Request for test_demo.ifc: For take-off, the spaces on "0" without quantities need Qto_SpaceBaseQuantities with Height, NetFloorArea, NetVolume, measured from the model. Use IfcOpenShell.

First a look at what the model holds.

```python
import ifcopenshell
import ifcopenshell.util.element
import ifcopenshell.util.unit

model = ifcopenshell.open("test_demo.ifc")
print(model.schema)
for unit_type in ("LENGTHUNIT", "AREAUNIT", "VOLUMEUNIT"):
    print(unit_type, ifcopenshell.util.unit.calculate_unit_scale(model, unit_type))
storey = next(s for s in model.by_type("IfcBuildingStorey") if s.Name == "0")
spaces = [e for e in ifcopenshell.util.element.get_decomposition(storey) if e.is_a("IfcSpace")]
for e in sorted(spaces, key=lambda e: e.id()):
    print(e.id(), e.is_a(), e.Name, list(ifcopenshell.util.element.get_psets(e, qtos_only=True)), sep=" | ")
```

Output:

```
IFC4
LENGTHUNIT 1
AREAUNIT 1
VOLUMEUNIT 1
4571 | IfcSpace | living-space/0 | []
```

```python
import ifcopenshell
import ifcopenshell.api.pset
import ifcopenshell.geom
import ifcopenshell.util.element
import ifcopenshell.util.shape
import ifcopenshell.util.unit

model = ifcopenshell.open("test_demo.ifc")
unit_scale = ifcopenshell.util.unit.calculate_unit_scale(model)
area_scale = ifcopenshell.util.unit.calculate_unit_scale(model, "AREAUNIT")
volume_scale = ifcopenshell.util.unit.calculate_unit_scale(model, "VOLUMEUNIT")
settings = ifcopenshell.geom.settings()

storey = next(s for s in model.by_type("IfcBuildingStorey") if s.Name == "0")
spaces = [e for e in ifcopenshell.util.element.get_decomposition(storey) if e.is_a("IfcSpace")]

for e in sorted(spaces, key=lambda e: e.id()):
    if ifcopenshell.util.element.get_psets(e, qtos_only=True, should_inherit=False):
        continue
    # Geometry comes back in metres, in the element's own axes.
    shape = ifcopenshell.geom.create_shape(settings, e)
    values = {
        "Height": ifcopenshell.util.shape.get_z(shape.geometry) / unit_scale,
        "NetFloorArea": ifcopenshell.util.shape.get_footprint_area(shape.geometry) / area_scale,
        "NetVolume": ifcopenshell.util.shape.get_volume(shape.geometry) / volume_scale,
    }
    qto = ifcopenshell.api.pset.add_qto(model, product=e, name="Qto_SpaceBaseQuantities")
    ifcopenshell.api.pset.edit_qto(model, qto=qto, properties=values)
    print(e.id(), {k: round(v, 3) for k, v in values.items()})

model.write("test_demo_edited.ifc")
```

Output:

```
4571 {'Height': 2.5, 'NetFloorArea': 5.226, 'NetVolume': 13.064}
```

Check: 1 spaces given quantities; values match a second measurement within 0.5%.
